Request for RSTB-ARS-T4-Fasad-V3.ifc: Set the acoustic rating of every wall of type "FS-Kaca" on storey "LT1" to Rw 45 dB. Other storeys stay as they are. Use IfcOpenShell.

First a look at what the model holds.

```python
import ifcopenshell
import ifcopenshell.util.element

model = ifcopenshell.open("RSTB-ARS-T4-Fasad-V3.ifc")
print(model.schema)
storey = next(s for s in model.by_type("IfcBuildingStorey") if s.Name == "LT1")
walls = [e for e in ifcopenshell.util.element.get_decomposition(storey) if e.is_a("IfcWall")]
seen = {}
for e in walls:
    element_type = ifcopenshell.util.element.get_type(e)
    key = (element_type.Name if element_type != e and element_type else None, ifcopenshell.util.element.get_pset(e, "Pset_WallCommon", "AcousticRating"))
    seen[key] = seen.get(key, 0) + 1
for (name, value), count in sorted(seen.items(), key=str):
    print(count, "x", name, "|", value)
```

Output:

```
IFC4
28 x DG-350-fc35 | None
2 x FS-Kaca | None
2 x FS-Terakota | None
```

```python
import ifcopenshell
import ifcopenshell.api.pset
import ifcopenshell.util.element

model = ifcopenshell.open("RSTB-ARS-T4-Fasad-V3.ifc")

storey = next(s for s in model.by_type("IfcBuildingStorey") if s.Name == "LT1")
walls = [e for e in ifcopenshell.util.element.get_decomposition(storey) if e.is_a("IfcWall")]

count = 0
for e in walls:
    element_type = ifcopenshell.util.element.get_type(e)
    if element_type in (None, e) or element_type.Name != "FS-Kaca":
        continue
    # add_pset returns the element's existing set when there is one.
    pset = ifcopenshell.api.pset.add_pset(model, product=e, name="Pset_WallCommon")
    ifcopenshell.api.pset.edit_pset(model, pset=pset, properties={"AcousticRating": "Rw 45 dB"})
    count += 1

print(count, "walls updated")

model.write("RSTB-ARS-T4-Fasad-V3-out.ifc")
```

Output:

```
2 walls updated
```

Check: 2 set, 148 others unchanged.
